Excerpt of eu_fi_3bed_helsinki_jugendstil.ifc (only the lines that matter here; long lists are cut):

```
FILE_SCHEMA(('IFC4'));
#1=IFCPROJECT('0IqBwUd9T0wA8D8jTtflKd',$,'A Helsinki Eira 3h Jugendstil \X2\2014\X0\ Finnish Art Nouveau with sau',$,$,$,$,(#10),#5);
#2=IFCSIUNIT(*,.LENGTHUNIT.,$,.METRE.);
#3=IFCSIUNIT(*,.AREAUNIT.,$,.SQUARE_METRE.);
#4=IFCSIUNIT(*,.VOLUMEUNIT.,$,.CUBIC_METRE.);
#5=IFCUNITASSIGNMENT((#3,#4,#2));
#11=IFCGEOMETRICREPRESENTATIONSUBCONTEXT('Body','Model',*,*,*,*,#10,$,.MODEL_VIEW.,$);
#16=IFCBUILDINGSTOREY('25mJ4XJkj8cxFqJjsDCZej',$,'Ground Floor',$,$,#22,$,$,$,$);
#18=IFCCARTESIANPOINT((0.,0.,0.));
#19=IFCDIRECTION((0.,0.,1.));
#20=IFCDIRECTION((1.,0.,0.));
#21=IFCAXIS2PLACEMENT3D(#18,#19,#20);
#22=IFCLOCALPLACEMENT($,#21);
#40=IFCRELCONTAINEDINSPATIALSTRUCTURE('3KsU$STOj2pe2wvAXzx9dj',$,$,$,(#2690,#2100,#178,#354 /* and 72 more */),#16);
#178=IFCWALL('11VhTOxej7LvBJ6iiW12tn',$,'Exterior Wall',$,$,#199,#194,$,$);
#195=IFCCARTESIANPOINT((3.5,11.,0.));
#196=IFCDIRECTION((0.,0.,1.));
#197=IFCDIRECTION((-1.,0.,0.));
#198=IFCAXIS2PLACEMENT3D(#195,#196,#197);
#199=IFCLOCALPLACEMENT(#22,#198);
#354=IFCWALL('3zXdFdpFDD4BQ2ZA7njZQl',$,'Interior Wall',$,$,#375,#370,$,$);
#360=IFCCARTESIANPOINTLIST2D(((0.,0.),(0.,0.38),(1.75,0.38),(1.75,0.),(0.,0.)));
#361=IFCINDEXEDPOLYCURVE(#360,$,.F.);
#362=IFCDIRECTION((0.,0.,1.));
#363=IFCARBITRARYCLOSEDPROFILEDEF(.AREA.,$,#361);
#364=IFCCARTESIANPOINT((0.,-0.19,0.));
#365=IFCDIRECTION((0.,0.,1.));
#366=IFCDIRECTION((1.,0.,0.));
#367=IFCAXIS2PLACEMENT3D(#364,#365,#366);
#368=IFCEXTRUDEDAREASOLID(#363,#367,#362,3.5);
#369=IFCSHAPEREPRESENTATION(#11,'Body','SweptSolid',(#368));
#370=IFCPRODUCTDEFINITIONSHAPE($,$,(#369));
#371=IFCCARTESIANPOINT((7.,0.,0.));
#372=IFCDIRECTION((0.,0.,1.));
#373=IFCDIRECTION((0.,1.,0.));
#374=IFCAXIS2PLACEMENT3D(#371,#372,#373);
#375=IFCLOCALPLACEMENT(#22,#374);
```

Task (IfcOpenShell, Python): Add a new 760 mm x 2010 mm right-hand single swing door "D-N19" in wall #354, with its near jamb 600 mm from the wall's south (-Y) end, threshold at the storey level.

```python
import numpy as np
import ifcopenshell
import ifcopenshell.api.feature
import ifcopenshell.api.geometry
import ifcopenshell.api.root
import ifcopenshell.api.spatial
import ifcopenshell.geom
import ifcopenshell.util.element
import ifcopenshell.util.placement
import ifcopenshell.util.representation
import ifcopenshell.util.shape
import ifcopenshell.util.unit

model = ifcopenshell.open("eu_fi_3bed_helsinki_jugendstil.ifc")
unit_scale = ifcopenshell.util.unit.calculate_unit_scale(model)
settings = ifcopenshell.geom.settings()


def volume(element):
    """Net volume in cubic metres, openings subtracted."""
    shape = ifcopenshell.geom.create_shape(settings, element)
    return ifcopenshell.util.shape.get_volume(shape.geometry)


wall = model.by_id(354)
storey = ifcopenshell.util.element.get_container(wall, ifc_class="IfcBuildingStorey")
context = ifcopenshell.util.representation.get_context(model, "Model", "Body", "MODEL_VIEW")
before = volume(wall)

width, height, from_end, sill = 0.76, 2.01, 0.6, 0.0  # metres

# The wall runs along its own X axis, and the end named is its -X end.
wall_shape = ifcopenshell.geom.create_shape(settings, wall)
x, y, z = ifcopenshell.util.shape.get_vertices(wall_shape.geometry).T
start = x.min() + from_end
face, thickness = float(y.min()), float(y.max() - y.min())
wall_matrix = ifcopenshell.util.placement.get_local_placement(wall.ObjectPlacement)
level = ifcopenshell.util.placement.get_local_placement(storey.ObjectPlacement)[2, 3]


def in_wall(x, y):
    """Placement at x, y metres in the wall's axes, at sill height."""
    matrix = wall_matrix.copy()
    matrix[:, 3] = wall_matrix @ np.array([x / unit_scale, y / unit_scale, 0.0, 1.0])
    matrix[2, 3] = level + sill / unit_scale
    return matrix


# Opening: a box that overshoots both wall faces by 50 mm.
opening = ifcopenshell.api.root.create_entity(model, ifc_class="IfcOpeningElement", predefined_type="OPENING")
box = ifcopenshell.api.geometry.add_wall_representation(
    model, context=context, length=width, height=height, thickness=thickness + 0.1
)
ifcopenshell.api.geometry.assign_representation(model, product=opening, representation=box)
ifcopenshell.api.geometry.edit_object_placement(model, product=opening, matrix=in_wall(start, face - 0.05), is_si=False)
ifcopenshell.api.feature.add_feature(model, feature=opening, element=wall)

door = ifcopenshell.api.root.create_entity(model, ifc_class="IfcDoor", name="D-N19", predefined_type="DOOR")
door.OverallWidth, door.OverallHeight = width / unit_scale, height / unit_scale
door.OperationType = "SINGLE_SWING_RIGHT"
body = ifcopenshell.api.geometry.add_door_representation(
    model,
    context=context,
    overall_width=door.OverallWidth,
    overall_height=door.OverallHeight,
    operation_type="SINGLE_SWING_RIGHT",
    lining_properties={"LiningDepth": thickness / unit_scale, "ThresholdDepth": thickness / unit_scale},
)
ifcopenshell.api.geometry.assign_representation(model, product=door, representation=body)
ifcopenshell.api.spatial.assign_container(model, products=[door], relating_structure=storey)
ifcopenshell.api.feature.add_filling(model, opening=opening, element=door)

# The lining spans the wall, so the door starts at the wall face.
ifcopenshell.api.geometry.edit_object_placement(model, product=door, matrix=in_wall(start, face), is_si=False)

after = volume(wall)

print(f"wall volume {before:.3f} -> {after:.3f} m3")

model.write("eu_fi_3bed_helsinki_jugendstil_v2.ifc")
```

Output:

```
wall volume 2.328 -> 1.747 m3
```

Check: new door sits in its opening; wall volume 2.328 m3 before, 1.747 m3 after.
